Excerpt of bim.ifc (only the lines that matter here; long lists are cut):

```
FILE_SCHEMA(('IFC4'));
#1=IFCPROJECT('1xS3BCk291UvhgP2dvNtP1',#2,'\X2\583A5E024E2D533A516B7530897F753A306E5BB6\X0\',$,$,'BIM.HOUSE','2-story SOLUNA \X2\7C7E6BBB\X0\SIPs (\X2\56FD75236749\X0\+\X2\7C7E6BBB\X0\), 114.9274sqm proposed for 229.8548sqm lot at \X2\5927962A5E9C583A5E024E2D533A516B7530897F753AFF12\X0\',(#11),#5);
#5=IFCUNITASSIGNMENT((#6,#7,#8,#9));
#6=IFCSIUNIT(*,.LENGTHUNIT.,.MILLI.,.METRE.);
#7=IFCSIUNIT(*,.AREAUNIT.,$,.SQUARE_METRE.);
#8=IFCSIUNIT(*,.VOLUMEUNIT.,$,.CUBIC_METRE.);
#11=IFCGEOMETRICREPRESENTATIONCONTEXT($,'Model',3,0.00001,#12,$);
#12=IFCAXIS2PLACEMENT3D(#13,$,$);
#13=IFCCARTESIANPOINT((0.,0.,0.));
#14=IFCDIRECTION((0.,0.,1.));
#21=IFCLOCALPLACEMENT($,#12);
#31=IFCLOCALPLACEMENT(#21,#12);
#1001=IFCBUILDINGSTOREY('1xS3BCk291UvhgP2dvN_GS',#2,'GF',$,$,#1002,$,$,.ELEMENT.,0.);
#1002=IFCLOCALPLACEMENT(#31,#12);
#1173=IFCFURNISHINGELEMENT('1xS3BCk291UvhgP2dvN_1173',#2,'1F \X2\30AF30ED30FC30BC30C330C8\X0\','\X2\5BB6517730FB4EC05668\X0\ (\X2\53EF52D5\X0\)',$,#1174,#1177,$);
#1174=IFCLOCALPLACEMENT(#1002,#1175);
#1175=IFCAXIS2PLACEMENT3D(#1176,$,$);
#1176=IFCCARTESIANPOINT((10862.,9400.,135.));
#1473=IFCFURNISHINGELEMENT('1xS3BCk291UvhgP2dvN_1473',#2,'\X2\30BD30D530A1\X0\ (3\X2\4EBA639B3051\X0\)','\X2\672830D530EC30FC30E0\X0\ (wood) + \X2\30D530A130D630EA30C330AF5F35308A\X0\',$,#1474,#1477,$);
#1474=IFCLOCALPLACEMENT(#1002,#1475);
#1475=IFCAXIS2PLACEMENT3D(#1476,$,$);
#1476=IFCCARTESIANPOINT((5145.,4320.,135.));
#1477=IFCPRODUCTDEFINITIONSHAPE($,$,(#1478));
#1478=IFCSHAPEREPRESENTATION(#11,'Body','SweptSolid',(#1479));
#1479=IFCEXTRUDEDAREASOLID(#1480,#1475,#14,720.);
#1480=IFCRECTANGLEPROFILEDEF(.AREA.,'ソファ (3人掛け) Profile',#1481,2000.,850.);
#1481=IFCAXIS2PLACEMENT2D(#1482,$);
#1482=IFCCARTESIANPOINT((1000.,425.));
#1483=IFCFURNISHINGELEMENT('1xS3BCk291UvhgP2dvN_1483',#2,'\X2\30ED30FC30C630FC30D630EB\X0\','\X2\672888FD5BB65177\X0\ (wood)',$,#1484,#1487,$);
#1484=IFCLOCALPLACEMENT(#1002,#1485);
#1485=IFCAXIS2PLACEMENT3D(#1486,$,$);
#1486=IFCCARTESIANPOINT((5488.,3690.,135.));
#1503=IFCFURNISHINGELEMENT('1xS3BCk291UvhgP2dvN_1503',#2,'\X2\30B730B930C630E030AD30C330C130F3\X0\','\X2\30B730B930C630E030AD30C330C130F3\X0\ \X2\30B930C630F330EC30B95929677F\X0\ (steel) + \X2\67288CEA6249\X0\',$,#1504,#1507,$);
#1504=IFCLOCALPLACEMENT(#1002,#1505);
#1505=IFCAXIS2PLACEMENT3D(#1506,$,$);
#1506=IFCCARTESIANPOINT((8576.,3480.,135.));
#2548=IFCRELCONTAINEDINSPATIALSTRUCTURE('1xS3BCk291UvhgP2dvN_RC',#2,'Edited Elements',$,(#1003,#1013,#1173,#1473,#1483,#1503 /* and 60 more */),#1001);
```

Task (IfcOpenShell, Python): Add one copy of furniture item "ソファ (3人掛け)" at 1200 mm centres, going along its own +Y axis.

```python
import ifcopenshell
import ifcopenshell.api.geometry
import ifcopenshell.api.root
import ifcopenshell.util.element
import ifcopenshell.util.placement

model = ifcopenshell.open("bim.ifc")


def reuse_history(source, copy):
    """copy_class also copies each property set's owner history, people and application; keep the originals."""
    for rel in copy.IsDefinedBy:
        if rel.is_a("IfcRelDefinesByProperties") and (history := rel.RelatingPropertyDefinition.OwnerHistory):
            rel.RelatingPropertyDefinition.OwnerHistory = source.OwnerHistory
            ifcopenshell.util.element.remove_deep2(model, history)


source = model.by_id(1473)
base = ifcopenshell.util.placement.get_local_placement(source.ObjectPlacement)
step = base[:3, 1] * 1200.0

for i in range(1, 2):
    copy = ifcopenshell.api.root.copy_class(model, product=source)
    copy.Representation = ifcopenshell.util.element.copy_deep(
        model, source.Representation, exclude=["IfcGeometricRepresentationContext", "IfcRepresentationMap"]
    )
    reuse_history(source, copy)
    matrix = base.copy()
    matrix[:3, 3] += i * step
    print("added at", matrix[:3, 3].round(3) + 0.0)
    ifcopenshell.api.geometry.edit_object_placement(model, product=copy, matrix=matrix, is_si=False)

model.write("bim_v2.ifc")
```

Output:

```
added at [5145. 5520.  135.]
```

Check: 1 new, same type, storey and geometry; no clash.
